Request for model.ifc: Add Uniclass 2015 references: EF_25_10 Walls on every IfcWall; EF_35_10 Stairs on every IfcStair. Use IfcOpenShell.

First a look at what the model holds.

```python
import ifcopenshell

model = ifcopenshell.open("model.ifc")
print(model.schema)
print("classifications:", [c.Name for c in model.by_type("IfcClassification")])
for ifc_class in ("IfcDoor", "IfcRoof", "IfcStair", "IfcWall", "IfcWindow"):
    print(ifc_class, len(model.by_type(ifc_class)))
```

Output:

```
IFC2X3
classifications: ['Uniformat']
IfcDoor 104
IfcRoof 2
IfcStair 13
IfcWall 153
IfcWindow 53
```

```python
import ifcopenshell
import ifcopenshell.api.classification

model = ifcopenshell.open("model.ifc")

# IFC2X3 requires Source and Edition and has no link from the project to the system.
system = model.create_entity("IfcClassification", Source="NBS", Edition="2015", Name="Uniclass 2015")

codes = {
    "IfcWall": ("EF_25_10", "Walls"),
    "IfcStair": ("EF_35_10", "Stairs"),
}
for ifc_class, (code, name) in codes.items():
    products = model.by_type(ifc_class)
    ifcopenshell.api.classification.add_reference(
        model, products=products, classification=system, identification=code, name=name
    )
    print(code, len(products))

model.write("model_rev.ifc")
```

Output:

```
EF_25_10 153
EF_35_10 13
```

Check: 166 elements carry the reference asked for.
